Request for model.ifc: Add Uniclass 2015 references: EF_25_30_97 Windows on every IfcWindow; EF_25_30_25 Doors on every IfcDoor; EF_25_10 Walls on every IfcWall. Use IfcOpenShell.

First a look at what the model holds.

```python
import ifcopenshell

model = ifcopenshell.open("model.ifc")
print(model.schema)
print("classifications:", [c.Name for c in model.by_type("IfcClassification")])
for ifc_class in ("IfcDoor", "IfcRoof", "IfcStair", "IfcWall", "IfcWindow"):
    print(ifc_class, len(model.by_type(ifc_class)))
```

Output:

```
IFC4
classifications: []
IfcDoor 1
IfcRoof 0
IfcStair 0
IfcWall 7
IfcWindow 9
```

```python
import ifcopenshell
import ifcopenshell.api.classification

model = ifcopenshell.open("model.ifc")

system = ifcopenshell.api.classification.add_classification(model, classification="Uniclass 2015")

codes = {
    "IfcWindow": ("EF_25_30_97", "Windows"),
    "IfcDoor": ("EF_25_30_25", "Doors"),
    "IfcWall": ("EF_25_10", "Walls"),
}
for ifc_class, (code, name) in codes.items():
    products = model.by_type(ifc_class)
    ifcopenshell.api.classification.add_reference(
        model, products=products, classification=system, identification=code, name=name
    )
    print(code, len(products))

model.write("model_rev.ifc")
```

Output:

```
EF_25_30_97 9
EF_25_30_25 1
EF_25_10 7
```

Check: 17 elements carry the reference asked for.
